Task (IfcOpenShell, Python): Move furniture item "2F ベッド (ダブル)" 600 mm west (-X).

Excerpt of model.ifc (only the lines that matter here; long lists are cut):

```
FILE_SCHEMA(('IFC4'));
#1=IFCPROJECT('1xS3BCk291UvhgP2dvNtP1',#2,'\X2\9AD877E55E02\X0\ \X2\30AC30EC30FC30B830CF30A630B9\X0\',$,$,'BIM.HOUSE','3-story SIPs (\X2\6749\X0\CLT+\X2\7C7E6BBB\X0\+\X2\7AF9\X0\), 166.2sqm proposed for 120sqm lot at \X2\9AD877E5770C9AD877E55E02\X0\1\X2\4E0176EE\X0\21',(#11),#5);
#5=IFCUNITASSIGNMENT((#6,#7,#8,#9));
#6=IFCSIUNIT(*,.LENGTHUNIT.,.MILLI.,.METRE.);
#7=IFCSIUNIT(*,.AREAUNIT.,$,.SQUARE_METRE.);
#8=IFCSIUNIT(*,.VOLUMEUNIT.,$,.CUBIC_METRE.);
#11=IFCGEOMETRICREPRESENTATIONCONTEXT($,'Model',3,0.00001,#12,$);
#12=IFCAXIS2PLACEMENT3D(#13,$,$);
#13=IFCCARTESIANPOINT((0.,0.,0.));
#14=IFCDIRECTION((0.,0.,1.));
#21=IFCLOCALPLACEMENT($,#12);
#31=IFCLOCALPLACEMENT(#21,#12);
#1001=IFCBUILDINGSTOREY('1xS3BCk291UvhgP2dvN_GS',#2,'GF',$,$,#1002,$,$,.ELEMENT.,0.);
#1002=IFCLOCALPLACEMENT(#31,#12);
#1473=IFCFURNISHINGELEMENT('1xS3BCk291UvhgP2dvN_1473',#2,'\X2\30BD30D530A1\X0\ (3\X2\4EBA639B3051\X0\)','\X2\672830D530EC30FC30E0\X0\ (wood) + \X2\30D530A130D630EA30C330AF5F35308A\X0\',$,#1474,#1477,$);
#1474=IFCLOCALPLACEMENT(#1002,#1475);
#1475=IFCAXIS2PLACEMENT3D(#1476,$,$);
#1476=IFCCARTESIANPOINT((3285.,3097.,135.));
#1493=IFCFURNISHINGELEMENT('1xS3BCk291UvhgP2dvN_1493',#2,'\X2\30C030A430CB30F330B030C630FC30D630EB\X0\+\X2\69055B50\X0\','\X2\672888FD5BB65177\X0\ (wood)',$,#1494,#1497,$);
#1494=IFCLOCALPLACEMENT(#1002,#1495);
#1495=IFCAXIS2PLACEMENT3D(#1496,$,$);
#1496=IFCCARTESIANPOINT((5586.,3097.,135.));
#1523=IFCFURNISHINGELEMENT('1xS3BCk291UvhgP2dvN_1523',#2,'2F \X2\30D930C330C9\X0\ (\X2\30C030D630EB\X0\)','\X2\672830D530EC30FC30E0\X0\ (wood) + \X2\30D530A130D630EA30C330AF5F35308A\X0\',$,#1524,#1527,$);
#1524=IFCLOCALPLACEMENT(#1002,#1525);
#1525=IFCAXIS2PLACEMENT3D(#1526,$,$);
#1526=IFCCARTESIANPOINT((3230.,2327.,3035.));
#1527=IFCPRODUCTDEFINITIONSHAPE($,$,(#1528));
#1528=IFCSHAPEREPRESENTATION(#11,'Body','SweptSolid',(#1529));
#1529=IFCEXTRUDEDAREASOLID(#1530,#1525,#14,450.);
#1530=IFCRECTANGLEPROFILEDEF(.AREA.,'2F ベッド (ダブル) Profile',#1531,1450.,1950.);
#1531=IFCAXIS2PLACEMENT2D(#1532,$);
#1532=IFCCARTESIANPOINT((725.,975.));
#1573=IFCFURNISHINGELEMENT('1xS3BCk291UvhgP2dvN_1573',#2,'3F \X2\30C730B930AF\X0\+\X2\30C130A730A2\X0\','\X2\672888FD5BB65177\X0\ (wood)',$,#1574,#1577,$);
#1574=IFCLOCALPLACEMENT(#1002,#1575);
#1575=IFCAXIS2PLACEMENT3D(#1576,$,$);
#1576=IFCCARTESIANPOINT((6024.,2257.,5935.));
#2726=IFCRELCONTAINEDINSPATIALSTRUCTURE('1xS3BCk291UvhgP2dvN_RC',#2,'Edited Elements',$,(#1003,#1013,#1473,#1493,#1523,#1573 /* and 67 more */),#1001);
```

```python
import ifcopenshell
import ifcopenshell.api.geometry
import ifcopenshell.util.placement

model = ifcopenshell.open("model.ifc")

item = model.by_guid("1xS3BCk291UvhgP2dvN_1523")
matrix = ifcopenshell.util.placement.get_local_placement(item.ObjectPlacement)
matrix[0, 3] -= 600.0
ifcopenshell.api.geometry.edit_object_placement(model, product=item, matrix=matrix, is_si=False)

print(ifcopenshell.util.placement.get_local_placement(item.ObjectPlacement).round(3) + 0.0)

model.write("model_edited.ifc")
```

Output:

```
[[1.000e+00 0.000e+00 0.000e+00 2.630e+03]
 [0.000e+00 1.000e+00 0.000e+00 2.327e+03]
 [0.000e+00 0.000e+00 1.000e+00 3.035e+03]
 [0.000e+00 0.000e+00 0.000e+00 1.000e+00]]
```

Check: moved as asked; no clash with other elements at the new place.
